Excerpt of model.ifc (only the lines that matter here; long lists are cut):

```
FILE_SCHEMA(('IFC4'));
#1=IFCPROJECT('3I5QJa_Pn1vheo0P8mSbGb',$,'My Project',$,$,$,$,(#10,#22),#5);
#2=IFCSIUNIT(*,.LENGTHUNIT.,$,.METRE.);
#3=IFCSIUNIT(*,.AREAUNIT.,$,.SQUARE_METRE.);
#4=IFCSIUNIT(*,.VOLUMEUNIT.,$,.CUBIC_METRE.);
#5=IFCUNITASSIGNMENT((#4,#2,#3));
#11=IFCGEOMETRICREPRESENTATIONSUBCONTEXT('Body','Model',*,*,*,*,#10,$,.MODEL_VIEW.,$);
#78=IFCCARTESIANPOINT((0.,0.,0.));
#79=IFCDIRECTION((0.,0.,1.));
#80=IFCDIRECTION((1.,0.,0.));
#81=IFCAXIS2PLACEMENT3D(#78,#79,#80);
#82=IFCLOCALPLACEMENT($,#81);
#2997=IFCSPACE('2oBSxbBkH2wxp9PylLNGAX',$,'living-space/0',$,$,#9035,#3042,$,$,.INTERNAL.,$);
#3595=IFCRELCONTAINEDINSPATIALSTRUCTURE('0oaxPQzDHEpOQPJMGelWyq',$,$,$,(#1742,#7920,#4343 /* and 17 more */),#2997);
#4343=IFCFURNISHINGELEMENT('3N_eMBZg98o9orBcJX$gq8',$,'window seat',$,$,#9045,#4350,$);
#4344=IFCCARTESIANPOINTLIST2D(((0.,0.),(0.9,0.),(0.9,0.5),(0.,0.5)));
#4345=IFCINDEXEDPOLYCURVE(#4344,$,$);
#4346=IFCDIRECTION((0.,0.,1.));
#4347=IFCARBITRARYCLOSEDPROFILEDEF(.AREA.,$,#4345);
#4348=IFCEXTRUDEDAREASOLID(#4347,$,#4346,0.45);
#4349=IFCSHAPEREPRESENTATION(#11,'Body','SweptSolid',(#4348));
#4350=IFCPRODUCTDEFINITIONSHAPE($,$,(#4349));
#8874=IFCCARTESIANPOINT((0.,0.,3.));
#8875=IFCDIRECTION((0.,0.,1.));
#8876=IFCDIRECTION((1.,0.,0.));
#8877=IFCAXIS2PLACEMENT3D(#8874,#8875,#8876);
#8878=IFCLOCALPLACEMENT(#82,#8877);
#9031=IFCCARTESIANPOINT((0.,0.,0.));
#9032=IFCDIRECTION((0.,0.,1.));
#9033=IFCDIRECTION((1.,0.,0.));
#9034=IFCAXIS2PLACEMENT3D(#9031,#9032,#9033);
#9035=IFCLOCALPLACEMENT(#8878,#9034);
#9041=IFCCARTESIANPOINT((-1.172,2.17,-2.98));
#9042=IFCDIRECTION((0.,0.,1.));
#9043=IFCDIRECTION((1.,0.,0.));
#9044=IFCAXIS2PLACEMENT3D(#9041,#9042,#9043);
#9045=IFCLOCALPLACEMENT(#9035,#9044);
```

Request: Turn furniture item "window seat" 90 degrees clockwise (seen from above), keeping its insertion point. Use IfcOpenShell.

```python
import ifcopenshell
import ifcopenshell.api.geometry
import ifcopenshell.util.placement

model = ifcopenshell.open("model.ifc")

item = model.by_guid("3N_eMBZg98o9orBcJX$gq8")
matrix = ifcopenshell.util.placement.get_local_placement(item.ObjectPlacement)
matrix = matrix @ ifcopenshell.util.placement.rotation(-90, "Z")
ifcopenshell.api.geometry.edit_object_placement(model, product=item, matrix=matrix, is_si=False)

print(ifcopenshell.util.placement.get_local_placement(item.ObjectPlacement).round(3) + 0.0)

model.write("model_updated.ifc")
```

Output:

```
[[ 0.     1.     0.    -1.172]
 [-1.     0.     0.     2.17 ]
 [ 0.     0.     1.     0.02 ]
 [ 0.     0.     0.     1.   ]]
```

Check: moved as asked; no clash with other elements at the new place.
